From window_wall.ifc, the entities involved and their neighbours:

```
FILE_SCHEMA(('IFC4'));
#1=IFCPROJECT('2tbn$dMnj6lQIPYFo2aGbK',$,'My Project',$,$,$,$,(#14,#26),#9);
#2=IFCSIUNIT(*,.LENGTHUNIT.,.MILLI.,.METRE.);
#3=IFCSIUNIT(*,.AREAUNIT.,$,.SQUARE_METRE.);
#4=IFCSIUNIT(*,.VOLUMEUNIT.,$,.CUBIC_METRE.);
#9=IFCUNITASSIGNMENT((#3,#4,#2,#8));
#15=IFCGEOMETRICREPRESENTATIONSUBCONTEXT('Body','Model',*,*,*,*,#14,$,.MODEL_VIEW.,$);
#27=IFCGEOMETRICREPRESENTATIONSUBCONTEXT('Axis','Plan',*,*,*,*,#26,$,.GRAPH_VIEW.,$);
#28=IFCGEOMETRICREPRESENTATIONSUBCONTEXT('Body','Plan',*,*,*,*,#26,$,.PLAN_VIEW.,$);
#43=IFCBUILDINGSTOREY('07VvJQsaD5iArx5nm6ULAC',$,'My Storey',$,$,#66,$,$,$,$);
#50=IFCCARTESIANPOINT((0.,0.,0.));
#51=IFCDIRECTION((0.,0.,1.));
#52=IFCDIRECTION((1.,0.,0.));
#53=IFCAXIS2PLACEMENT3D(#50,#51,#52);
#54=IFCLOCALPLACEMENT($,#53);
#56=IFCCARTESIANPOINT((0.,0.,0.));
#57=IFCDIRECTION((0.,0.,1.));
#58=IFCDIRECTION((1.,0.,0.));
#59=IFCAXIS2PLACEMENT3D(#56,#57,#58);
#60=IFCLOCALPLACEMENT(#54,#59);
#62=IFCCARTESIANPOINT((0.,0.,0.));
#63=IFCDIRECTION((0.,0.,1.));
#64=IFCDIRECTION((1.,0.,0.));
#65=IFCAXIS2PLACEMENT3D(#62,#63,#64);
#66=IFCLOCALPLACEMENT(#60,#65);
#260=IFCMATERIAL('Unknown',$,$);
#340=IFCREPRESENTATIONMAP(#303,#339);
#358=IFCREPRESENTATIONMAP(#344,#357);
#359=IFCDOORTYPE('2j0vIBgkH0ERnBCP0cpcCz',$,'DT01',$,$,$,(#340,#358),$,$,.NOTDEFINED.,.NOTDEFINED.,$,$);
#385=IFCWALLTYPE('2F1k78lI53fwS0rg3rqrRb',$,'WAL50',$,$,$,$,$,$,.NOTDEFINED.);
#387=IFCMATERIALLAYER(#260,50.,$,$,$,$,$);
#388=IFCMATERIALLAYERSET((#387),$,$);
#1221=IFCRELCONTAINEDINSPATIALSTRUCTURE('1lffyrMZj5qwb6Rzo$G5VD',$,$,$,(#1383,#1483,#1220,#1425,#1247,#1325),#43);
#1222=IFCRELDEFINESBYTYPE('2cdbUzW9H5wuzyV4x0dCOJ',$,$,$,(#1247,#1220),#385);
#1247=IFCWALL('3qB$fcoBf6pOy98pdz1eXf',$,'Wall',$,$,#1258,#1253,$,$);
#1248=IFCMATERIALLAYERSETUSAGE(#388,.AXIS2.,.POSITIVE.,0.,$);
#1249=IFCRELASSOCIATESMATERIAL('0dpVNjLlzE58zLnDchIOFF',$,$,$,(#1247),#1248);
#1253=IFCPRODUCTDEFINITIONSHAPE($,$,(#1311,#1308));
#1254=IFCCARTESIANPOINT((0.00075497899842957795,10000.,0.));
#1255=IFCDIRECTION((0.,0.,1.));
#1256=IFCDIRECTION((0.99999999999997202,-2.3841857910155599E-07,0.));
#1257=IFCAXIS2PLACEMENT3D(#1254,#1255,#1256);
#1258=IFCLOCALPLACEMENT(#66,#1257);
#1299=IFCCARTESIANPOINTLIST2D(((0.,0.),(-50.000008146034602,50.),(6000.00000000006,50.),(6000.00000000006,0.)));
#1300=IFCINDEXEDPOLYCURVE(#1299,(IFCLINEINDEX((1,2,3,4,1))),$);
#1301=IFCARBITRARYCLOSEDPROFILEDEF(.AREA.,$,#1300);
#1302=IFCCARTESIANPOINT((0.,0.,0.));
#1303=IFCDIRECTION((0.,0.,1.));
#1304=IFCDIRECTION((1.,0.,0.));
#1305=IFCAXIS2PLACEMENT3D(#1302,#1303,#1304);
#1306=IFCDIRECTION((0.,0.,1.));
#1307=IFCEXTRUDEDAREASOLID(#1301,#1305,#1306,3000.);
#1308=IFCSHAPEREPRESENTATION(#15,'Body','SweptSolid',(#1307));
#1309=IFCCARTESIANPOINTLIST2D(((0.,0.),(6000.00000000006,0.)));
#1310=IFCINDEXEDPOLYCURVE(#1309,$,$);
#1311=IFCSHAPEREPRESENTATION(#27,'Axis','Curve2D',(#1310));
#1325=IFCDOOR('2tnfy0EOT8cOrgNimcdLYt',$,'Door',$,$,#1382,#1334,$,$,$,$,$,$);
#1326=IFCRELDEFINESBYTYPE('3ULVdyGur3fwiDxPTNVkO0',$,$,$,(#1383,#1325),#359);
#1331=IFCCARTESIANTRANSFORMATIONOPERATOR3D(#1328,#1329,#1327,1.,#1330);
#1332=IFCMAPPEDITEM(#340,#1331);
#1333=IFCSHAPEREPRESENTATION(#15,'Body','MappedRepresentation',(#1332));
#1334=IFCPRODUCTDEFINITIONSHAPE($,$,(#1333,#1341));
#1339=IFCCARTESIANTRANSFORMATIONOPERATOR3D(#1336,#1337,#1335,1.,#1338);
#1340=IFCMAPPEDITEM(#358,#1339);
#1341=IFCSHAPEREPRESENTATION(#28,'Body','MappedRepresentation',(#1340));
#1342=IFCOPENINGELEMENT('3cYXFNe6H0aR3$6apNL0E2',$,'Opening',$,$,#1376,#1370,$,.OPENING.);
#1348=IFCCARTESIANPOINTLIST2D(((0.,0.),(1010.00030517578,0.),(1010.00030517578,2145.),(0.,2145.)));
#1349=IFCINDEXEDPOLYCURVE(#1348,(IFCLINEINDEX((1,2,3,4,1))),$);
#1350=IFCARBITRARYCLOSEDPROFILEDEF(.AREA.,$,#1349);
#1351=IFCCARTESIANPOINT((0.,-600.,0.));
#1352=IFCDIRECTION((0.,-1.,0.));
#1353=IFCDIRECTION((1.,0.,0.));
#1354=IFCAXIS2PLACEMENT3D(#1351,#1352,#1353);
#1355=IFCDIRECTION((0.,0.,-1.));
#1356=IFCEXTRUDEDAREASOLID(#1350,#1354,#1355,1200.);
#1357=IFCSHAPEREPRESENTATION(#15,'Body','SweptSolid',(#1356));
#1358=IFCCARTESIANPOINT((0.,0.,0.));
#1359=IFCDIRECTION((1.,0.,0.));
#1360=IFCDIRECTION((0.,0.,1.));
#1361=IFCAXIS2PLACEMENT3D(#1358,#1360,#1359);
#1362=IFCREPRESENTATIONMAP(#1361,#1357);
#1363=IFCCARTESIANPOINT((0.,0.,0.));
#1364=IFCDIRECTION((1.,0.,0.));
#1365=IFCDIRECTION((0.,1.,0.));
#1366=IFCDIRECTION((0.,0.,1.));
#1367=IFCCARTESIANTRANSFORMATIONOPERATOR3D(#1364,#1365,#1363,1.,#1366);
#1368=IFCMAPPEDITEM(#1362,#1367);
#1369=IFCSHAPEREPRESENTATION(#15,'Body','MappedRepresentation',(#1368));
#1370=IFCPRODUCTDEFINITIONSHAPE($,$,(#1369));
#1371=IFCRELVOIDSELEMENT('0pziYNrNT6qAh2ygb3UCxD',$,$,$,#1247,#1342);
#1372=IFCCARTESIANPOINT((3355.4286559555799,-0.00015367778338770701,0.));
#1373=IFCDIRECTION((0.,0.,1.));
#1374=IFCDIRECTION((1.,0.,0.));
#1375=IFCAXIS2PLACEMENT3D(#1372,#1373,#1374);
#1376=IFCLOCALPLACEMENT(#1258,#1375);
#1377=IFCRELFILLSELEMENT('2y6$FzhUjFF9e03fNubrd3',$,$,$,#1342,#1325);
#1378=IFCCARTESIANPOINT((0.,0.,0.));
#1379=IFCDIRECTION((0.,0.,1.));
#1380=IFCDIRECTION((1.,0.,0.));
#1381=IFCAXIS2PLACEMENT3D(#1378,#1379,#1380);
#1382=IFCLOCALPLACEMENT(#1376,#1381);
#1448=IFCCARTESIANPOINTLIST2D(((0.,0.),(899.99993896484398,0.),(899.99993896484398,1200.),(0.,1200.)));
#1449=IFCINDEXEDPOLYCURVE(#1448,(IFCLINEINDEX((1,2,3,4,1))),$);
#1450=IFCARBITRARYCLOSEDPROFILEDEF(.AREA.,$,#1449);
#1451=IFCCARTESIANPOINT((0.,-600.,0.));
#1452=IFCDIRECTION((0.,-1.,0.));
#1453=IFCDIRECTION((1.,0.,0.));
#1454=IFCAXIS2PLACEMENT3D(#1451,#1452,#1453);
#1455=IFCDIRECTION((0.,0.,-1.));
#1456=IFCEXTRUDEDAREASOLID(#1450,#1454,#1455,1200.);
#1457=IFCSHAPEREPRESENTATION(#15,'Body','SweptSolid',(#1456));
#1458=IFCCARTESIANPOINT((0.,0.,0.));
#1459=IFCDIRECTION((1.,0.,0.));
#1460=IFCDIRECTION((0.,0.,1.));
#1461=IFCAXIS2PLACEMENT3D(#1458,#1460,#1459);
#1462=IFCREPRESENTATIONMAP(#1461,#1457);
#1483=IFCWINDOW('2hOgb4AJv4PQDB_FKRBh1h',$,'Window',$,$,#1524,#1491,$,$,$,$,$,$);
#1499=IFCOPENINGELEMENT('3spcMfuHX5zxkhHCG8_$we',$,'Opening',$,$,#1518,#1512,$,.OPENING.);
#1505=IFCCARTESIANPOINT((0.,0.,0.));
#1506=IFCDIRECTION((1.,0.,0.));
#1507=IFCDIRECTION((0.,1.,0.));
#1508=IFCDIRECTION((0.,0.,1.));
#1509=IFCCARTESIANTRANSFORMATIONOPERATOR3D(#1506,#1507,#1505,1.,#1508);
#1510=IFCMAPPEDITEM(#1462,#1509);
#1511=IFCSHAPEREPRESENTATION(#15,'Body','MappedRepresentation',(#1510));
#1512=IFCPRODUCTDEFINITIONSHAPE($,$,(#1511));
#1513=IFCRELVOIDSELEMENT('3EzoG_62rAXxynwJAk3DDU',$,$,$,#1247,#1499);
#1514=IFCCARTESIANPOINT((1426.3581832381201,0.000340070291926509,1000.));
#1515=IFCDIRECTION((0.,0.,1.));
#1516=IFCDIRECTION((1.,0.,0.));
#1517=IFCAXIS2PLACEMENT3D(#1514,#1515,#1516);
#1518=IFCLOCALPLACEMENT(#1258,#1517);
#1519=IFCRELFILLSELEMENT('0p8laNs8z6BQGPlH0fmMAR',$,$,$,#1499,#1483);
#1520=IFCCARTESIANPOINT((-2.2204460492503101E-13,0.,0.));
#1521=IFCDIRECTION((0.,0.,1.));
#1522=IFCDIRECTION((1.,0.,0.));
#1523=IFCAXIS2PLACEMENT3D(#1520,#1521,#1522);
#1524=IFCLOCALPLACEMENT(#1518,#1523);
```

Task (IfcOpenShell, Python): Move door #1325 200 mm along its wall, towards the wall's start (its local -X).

```python
import ifcopenshell
import ifcopenshell.api.geometry
import ifcopenshell.util.placement
import ifcopenshell.util.unit

model = ifcopenshell.open("window_wall.ifc")
unit_scale = ifcopenshell.util.unit.calculate_unit_scale(model)

door = model.by_id(1325)
opening = door.FillsVoids[0].RelatingOpeningElement
wall = opening.VoidsElements[0].RelatingBuildingElement

wall_matrix = ifcopenshell.util.placement.get_local_placement(wall.ObjectPlacement)
shift = wall_matrix[:3, 0] * -0.2 / unit_scale
before = ifcopenshell.util.placement.get_local_placement(door.ObjectPlacement)[:3, 3].copy()

# The door is placed relative to its opening, so it follows when the opening moves.
matrix = ifcopenshell.util.placement.get_local_placement(opening.ObjectPlacement)
matrix[:3, 3] += shift
ifcopenshell.api.geometry.edit_object_placement(
    model, product=opening, matrix=matrix, is_si=False, should_transform_children=True
)

after = ifcopenshell.util.placement.get_local_placement(door.ObjectPlacement)[:3, 3]
print("door moved by", (after - before).round(3) + 0.0)

model.write("window_wall_updated.ifc")
```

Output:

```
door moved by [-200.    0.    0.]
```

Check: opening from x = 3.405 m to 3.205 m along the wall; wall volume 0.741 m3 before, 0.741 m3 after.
